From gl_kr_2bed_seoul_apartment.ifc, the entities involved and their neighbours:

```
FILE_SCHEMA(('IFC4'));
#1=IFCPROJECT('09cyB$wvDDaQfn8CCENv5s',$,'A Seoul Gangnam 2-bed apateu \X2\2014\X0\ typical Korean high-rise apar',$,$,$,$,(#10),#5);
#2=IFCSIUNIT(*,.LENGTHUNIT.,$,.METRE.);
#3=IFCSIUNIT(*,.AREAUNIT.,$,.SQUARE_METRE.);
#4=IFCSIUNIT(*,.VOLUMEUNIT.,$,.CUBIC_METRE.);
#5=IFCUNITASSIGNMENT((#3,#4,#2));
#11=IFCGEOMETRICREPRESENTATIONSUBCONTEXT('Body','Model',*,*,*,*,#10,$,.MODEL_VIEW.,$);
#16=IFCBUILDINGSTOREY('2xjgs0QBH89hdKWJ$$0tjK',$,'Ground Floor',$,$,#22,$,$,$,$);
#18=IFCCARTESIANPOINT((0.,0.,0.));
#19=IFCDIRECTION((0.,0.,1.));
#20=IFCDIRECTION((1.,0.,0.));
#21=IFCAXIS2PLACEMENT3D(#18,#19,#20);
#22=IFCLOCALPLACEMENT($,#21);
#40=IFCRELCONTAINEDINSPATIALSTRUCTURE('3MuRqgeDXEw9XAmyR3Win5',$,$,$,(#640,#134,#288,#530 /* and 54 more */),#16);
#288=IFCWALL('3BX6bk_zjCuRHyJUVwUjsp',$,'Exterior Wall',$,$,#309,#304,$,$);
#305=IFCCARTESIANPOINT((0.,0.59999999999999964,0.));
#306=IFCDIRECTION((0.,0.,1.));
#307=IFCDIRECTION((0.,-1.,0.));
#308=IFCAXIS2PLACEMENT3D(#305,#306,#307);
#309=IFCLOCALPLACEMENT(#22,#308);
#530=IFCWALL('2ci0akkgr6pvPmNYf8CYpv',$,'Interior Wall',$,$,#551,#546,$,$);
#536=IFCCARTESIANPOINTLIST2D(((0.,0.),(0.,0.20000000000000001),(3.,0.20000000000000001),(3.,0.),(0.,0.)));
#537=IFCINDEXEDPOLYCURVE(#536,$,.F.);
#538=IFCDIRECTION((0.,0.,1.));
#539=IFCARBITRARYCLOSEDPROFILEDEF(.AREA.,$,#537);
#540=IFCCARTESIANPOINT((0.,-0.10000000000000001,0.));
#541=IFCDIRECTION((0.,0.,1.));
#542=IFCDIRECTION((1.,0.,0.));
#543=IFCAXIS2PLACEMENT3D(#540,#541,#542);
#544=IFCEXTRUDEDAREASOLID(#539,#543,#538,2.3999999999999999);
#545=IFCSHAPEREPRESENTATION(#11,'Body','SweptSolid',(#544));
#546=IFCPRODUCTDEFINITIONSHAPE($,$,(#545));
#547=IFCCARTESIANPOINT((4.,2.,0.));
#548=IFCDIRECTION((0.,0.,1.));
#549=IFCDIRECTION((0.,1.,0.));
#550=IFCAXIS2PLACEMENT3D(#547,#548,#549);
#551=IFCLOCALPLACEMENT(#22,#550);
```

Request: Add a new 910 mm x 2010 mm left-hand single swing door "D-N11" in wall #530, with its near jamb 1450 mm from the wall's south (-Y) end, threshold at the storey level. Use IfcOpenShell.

```python
import numpy as np
import ifcopenshell
import ifcopenshell.api.feature
import ifcopenshell.api.geometry
import ifcopenshell.api.root
import ifcopenshell.api.spatial
import ifcopenshell.geom
import ifcopenshell.util.element
import ifcopenshell.util.placement
import ifcopenshell.util.representation
import ifcopenshell.util.shape
import ifcopenshell.util.unit

model = ifcopenshell.open("gl_kr_2bed_seoul_apartment.ifc")
unit_scale = ifcopenshell.util.unit.calculate_unit_scale(model)
settings = ifcopenshell.geom.settings()


def volume(element):
    """Net volume in cubic metres, openings subtracted."""
    shape = ifcopenshell.geom.create_shape(settings, element)
    return ifcopenshell.util.shape.get_volume(shape.geometry)


wall = model.by_guid("2ci0akkgr6pvPmNYf8CYpv")
storey = ifcopenshell.util.element.get_container(wall, ifc_class="IfcBuildingStorey")
context = ifcopenshell.util.representation.get_context(model, "Model", "Body", "MODEL_VIEW")
before = volume(wall)

width, height, from_end, sill = 0.91, 2.01, 1.45, 0.0  # metres

# The wall runs along its own X axis, and the end named is its -X end.
wall_shape = ifcopenshell.geom.create_shape(settings, wall)
x, y, z = ifcopenshell.util.shape.get_vertices(wall_shape.geometry).T
start = x.min() + from_end
face, thickness = float(y.min()), float(y.max() - y.min())
wall_matrix = ifcopenshell.util.placement.get_local_placement(wall.ObjectPlacement)
level = ifcopenshell.util.placement.get_local_placement(storey.ObjectPlacement)[2, 3]


def in_wall(x, y):
    """Placement at x, y metres in the wall's axes, at sill height."""
    matrix = wall_matrix.copy()
    matrix[:, 3] = wall_matrix @ np.array([x / unit_scale, y / unit_scale, 0.0, 1.0])
    matrix[2, 3] = level + sill / unit_scale
    return matrix


# Opening: a box that overshoots both wall faces by 50 mm.
opening = ifcopenshell.api.root.create_entity(model, ifc_class="IfcOpeningElement", predefined_type="OPENING")
box = ifcopenshell.api.geometry.add_wall_representation(
    model, context=context, length=width, height=height, thickness=thickness + 0.1
)
ifcopenshell.api.geometry.assign_representation(model, product=opening, representation=box)
ifcopenshell.api.geometry.edit_object_placement(model, product=opening, matrix=in_wall(start, face - 0.05), is_si=False)
ifcopenshell.api.feature.add_feature(model, feature=opening, element=wall)

door = ifcopenshell.api.root.create_entity(model, ifc_class="IfcDoor", name="D-N11", predefined_type="DOOR")
door.OverallWidth, door.OverallHeight = width / unit_scale, height / unit_scale
door.OperationType = "SINGLE_SWING_LEFT"
body = ifcopenshell.api.geometry.add_door_representation(
    model,
    context=context,
    overall_width=door.OverallWidth,
    overall_height=door.OverallHeight,
    operation_type="SINGLE_SWING_LEFT",
    lining_properties={"LiningDepth": thickness / unit_scale, "ThresholdDepth": thickness / unit_scale},
)
ifcopenshell.api.geometry.assign_representation(model, product=door, representation=body)
ifcopenshell.api.spatial.assign_container(model, products=[door], relating_structure=storey)
ifcopenshell.api.feature.add_filling(model, opening=opening, element=door)

# The lining spans the wall, so the door starts at the wall face.
ifcopenshell.api.geometry.edit_object_placement(model, product=door, matrix=in_wall(start, face), is_si=False)

after = volume(wall)

print(f"wall volume {before:.3f} -> {after:.3f} m3")

model.write("gl_kr_2bed_seoul_apartment_edited.ifc")
```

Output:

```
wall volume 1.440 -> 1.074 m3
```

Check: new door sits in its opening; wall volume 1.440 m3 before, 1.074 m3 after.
